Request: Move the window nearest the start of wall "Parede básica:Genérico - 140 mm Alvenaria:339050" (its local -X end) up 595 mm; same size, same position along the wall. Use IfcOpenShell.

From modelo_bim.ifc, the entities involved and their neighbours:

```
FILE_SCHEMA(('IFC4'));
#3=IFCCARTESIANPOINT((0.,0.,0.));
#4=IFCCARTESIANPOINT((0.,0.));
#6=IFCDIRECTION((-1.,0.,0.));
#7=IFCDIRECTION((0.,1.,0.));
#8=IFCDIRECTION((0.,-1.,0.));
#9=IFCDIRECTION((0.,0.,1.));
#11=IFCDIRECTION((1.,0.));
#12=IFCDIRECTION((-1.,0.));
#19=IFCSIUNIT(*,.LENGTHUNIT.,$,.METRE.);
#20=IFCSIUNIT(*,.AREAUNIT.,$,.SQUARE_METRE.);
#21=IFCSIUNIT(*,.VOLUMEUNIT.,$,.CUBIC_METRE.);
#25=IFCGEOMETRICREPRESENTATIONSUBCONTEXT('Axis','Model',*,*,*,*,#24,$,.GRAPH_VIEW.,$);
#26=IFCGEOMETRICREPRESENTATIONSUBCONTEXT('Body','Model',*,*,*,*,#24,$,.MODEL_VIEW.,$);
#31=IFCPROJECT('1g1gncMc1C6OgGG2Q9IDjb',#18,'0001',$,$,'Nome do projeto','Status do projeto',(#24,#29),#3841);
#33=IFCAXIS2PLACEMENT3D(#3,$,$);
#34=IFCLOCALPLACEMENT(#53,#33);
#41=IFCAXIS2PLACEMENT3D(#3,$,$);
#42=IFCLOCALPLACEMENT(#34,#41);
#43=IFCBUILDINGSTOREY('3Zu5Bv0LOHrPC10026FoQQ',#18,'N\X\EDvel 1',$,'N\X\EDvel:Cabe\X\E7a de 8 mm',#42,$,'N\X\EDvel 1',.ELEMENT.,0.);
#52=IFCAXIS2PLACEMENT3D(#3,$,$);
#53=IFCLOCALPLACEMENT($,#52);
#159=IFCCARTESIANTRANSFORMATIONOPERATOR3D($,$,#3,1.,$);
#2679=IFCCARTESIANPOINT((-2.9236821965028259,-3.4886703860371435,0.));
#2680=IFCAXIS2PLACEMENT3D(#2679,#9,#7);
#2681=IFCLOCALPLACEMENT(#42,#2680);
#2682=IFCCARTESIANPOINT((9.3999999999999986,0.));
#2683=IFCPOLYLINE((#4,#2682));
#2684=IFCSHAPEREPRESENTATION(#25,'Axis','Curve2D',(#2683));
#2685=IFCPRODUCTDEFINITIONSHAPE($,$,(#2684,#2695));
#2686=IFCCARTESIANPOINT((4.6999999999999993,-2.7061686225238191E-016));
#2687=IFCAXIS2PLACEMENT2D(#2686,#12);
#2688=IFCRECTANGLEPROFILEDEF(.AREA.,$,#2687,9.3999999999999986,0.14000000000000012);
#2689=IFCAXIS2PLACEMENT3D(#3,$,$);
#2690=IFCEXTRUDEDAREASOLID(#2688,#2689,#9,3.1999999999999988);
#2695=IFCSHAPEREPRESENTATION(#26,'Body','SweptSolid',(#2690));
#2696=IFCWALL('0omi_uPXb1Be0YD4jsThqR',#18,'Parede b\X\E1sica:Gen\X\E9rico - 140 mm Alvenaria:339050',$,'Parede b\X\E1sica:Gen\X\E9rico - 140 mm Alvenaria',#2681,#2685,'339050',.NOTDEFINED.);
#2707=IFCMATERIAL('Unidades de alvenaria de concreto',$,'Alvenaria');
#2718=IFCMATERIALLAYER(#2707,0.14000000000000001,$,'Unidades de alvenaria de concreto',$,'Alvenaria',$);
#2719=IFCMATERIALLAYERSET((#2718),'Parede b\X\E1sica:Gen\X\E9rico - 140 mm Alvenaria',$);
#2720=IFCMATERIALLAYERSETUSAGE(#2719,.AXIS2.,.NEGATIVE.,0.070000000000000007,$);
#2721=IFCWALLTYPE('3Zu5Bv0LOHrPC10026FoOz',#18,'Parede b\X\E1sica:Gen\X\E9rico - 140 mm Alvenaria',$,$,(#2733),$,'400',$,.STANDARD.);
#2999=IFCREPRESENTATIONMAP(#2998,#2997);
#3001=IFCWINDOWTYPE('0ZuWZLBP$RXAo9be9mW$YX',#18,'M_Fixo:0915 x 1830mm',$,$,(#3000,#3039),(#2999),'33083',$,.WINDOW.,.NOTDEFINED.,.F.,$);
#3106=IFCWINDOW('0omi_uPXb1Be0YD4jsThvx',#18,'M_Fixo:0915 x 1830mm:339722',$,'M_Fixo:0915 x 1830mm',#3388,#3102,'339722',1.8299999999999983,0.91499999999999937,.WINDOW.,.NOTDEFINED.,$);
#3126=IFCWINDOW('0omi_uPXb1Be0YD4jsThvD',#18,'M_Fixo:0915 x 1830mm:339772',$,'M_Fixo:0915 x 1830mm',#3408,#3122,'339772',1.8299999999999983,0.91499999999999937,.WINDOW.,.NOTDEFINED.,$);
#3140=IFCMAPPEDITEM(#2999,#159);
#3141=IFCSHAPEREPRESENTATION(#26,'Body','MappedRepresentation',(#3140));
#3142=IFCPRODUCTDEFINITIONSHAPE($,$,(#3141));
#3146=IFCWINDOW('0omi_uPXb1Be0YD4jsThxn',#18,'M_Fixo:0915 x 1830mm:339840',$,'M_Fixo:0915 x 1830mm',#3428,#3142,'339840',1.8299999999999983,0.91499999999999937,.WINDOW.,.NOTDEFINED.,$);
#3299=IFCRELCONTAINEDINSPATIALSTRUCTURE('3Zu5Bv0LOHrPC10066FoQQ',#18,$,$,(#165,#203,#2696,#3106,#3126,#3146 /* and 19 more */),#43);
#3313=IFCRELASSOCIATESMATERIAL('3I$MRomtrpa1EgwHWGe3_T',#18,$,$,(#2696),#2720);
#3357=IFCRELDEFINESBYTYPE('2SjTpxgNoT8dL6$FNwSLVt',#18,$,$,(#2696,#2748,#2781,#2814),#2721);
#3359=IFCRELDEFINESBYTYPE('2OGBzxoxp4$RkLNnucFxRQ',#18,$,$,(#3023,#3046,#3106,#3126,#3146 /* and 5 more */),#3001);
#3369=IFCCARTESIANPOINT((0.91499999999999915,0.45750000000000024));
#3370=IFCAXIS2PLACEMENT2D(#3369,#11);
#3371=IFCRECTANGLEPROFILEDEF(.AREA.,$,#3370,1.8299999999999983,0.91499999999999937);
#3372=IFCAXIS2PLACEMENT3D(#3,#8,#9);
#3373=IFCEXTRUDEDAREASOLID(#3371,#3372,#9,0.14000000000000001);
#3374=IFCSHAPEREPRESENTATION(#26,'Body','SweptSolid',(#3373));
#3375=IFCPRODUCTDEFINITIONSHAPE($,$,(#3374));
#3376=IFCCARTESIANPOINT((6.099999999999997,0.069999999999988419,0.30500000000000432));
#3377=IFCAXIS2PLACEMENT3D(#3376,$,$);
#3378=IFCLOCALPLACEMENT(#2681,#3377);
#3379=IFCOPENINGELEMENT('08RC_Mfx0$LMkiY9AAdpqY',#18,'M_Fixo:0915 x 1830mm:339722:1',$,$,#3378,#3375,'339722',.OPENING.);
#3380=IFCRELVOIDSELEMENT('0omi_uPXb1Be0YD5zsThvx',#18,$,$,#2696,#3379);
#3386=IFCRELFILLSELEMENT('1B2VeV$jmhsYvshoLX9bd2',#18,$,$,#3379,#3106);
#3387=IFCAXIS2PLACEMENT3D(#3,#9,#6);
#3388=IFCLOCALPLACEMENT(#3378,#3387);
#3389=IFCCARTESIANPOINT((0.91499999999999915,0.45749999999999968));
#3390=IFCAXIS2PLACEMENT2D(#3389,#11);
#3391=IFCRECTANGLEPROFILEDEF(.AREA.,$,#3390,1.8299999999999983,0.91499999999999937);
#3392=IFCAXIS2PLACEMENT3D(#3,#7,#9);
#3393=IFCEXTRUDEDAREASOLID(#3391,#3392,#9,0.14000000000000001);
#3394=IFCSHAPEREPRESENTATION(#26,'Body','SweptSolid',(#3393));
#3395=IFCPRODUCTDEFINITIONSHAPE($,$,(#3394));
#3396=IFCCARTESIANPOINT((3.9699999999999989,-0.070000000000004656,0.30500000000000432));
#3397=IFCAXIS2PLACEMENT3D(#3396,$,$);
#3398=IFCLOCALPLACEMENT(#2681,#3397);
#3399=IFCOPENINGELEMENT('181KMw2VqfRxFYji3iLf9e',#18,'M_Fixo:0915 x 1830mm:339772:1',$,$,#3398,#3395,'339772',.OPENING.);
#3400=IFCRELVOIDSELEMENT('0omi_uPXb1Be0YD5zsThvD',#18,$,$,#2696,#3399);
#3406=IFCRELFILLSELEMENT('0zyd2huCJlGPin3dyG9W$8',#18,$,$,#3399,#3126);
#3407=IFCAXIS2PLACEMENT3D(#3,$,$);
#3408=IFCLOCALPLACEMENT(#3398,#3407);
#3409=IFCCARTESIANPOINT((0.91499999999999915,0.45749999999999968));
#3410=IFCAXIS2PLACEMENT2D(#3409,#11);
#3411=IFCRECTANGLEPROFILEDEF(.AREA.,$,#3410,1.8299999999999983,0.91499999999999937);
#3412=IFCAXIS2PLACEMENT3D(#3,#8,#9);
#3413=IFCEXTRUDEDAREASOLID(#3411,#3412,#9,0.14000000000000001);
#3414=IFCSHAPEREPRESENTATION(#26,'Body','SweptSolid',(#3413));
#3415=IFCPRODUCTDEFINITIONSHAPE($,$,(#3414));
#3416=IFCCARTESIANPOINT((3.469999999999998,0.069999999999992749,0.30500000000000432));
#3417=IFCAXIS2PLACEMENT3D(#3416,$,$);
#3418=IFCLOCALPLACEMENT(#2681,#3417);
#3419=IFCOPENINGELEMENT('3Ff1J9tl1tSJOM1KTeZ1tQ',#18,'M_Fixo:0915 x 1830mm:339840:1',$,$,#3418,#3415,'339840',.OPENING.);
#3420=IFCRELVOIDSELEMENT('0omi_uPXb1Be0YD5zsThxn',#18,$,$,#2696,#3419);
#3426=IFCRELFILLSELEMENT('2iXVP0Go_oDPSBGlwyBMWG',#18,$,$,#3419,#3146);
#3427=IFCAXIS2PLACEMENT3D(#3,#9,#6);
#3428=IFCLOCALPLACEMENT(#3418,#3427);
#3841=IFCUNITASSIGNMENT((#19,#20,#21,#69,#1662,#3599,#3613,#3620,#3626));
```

```python
import numpy as np
import ifcopenshell
import ifcopenshell.api.geometry
import ifcopenshell.util.placement
import ifcopenshell.util.unit

model = ifcopenshell.open("modelo_bim.ifc")
unit_scale = ifcopenshell.util.unit.calculate_unit_scale(model)

window = model.by_guid("0omi_uPXb1Be0YD4jsThxn")
opening = window.FillsVoids[0].RelatingOpeningElement
dz = 0.595 / unit_scale

shift = np.array([0.0, 0.0, dz])
# The window is placed relative to its opening, so it follows when the opening moves.
matrix = ifcopenshell.util.placement.get_local_placement(opening.ObjectPlacement)
matrix[:3, 3] += shift
ifcopenshell.api.geometry.edit_object_placement(
    model, product=opening, matrix=matrix, is_si=False, should_transform_children=True
)

print(f"moved by {dz * unit_scale:+.3f} m")

model.write("modelo_bim_edited.ifc")
```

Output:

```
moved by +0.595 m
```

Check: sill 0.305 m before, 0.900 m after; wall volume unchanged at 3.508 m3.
